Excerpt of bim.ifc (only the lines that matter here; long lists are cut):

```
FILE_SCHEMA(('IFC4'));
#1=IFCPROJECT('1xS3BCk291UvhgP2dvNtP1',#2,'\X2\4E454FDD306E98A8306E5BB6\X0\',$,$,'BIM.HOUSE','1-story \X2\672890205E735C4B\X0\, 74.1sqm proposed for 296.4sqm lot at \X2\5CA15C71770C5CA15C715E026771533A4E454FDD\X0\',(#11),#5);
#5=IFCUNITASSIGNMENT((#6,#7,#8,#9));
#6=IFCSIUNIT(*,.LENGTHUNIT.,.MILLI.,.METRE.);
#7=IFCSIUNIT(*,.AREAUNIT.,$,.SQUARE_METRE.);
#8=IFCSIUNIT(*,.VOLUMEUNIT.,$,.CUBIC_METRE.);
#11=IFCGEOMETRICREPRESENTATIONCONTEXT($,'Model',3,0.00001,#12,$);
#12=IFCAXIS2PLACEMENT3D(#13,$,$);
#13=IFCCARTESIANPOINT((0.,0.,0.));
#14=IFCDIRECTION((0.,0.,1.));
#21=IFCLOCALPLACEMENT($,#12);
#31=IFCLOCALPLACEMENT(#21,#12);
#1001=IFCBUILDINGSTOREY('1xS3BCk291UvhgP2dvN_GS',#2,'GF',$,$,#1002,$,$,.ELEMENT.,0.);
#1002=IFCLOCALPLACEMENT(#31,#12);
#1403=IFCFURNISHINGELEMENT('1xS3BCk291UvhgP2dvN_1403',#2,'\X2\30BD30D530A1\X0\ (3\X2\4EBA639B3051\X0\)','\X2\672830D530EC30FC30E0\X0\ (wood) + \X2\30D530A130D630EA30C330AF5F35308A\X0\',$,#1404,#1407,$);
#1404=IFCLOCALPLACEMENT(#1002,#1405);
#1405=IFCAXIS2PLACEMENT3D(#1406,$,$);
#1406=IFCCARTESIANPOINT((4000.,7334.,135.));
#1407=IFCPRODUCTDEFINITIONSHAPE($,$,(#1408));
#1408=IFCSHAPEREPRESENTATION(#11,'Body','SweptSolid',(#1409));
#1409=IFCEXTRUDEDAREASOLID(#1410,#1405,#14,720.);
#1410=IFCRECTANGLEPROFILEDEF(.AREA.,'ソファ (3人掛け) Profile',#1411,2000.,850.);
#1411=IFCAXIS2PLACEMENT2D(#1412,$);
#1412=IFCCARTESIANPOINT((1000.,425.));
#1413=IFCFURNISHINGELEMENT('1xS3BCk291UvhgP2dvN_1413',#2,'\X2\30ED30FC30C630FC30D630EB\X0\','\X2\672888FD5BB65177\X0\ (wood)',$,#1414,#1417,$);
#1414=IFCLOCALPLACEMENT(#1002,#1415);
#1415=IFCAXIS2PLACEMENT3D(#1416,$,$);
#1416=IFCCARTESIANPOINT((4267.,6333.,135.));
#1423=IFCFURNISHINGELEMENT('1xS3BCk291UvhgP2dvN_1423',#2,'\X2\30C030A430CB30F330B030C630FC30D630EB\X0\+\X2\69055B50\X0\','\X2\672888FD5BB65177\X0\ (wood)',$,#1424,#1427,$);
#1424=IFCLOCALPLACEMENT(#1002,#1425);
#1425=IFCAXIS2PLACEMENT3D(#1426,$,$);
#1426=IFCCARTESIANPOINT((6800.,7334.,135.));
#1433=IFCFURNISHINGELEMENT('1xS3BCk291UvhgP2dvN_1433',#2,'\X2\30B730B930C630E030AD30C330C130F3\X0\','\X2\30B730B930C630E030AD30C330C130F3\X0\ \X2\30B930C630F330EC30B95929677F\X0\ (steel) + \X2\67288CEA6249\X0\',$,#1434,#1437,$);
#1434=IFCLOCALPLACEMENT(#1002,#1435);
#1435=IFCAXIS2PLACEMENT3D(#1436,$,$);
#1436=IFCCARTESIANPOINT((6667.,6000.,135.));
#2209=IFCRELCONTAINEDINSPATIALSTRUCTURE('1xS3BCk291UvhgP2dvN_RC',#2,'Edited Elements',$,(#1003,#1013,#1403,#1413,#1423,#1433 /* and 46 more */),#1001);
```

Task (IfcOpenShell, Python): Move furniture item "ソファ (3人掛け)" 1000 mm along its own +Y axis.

```python
import ifcopenshell
import ifcopenshell.api.geometry
import ifcopenshell.util.placement
import ifcopenshell.util.unit

model = ifcopenshell.open("bim.ifc")
unit_scale = ifcopenshell.util.unit.calculate_unit_scale(model)

item = model.by_id(1403)
matrix = ifcopenshell.util.placement.get_local_placement(item.ObjectPlacement)
matrix[:3, 3] += matrix[:3, 1] * 1 / unit_scale
ifcopenshell.api.geometry.edit_object_placement(model, product=item, matrix=matrix, is_si=False)

print(ifcopenshell.util.placement.get_local_placement(item.ObjectPlacement).round(3) + 0.0)

model.write("bim_v2.ifc")
```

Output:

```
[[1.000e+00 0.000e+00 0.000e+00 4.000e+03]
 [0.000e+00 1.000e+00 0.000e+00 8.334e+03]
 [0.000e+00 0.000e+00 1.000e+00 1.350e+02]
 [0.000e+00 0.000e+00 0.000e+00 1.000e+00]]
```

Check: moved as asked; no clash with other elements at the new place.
